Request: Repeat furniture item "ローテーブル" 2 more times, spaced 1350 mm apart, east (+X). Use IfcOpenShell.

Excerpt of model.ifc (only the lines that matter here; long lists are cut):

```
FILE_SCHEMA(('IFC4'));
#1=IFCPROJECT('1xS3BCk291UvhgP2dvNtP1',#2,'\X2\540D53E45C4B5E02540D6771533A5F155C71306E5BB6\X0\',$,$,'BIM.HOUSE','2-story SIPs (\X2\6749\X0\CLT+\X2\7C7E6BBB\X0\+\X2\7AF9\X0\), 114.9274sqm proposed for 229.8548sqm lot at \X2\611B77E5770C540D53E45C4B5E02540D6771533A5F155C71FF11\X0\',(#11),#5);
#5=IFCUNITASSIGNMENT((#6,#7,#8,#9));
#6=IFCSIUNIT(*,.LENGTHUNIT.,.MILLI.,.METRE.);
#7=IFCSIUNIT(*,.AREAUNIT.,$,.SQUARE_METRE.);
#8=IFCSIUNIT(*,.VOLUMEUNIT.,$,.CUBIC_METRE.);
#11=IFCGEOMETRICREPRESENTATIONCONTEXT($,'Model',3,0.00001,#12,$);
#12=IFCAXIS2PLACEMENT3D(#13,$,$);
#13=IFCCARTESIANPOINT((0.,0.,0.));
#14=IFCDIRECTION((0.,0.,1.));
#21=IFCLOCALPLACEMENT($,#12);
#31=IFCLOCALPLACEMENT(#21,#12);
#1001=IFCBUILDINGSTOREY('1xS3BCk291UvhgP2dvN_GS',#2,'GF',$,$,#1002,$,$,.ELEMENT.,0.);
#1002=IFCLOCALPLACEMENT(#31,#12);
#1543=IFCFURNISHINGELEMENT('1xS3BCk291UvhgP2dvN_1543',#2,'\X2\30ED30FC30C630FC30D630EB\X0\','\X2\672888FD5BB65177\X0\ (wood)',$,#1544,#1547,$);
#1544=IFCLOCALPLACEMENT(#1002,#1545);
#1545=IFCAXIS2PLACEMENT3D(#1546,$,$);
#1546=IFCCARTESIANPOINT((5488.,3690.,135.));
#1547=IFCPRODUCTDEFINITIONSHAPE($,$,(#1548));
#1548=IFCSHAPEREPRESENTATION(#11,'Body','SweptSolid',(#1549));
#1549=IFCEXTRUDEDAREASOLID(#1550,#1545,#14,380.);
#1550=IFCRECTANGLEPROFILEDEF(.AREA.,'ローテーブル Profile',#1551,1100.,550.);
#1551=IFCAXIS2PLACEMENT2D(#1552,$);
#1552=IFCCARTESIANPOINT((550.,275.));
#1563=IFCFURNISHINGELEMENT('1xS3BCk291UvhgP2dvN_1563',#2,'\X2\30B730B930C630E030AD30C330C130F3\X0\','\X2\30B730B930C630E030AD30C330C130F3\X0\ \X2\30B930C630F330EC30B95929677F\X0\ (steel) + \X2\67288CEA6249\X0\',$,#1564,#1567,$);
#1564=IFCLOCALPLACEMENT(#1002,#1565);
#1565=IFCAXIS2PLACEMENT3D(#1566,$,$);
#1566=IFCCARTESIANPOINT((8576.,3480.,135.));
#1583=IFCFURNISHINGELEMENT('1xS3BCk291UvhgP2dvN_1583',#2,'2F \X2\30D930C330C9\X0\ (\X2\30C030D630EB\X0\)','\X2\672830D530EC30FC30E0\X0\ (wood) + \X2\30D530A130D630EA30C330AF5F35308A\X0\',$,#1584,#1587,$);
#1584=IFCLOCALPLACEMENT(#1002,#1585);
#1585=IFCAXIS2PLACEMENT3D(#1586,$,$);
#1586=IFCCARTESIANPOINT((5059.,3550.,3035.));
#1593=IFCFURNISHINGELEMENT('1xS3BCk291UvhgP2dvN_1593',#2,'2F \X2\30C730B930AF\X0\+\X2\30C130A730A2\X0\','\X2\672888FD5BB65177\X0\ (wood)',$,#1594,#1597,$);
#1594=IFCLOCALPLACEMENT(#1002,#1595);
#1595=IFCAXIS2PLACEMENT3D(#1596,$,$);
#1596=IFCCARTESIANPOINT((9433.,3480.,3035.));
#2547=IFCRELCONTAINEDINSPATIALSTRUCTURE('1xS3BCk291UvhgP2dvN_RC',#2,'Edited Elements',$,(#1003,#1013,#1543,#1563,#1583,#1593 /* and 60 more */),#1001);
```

```python
import numpy as np
import ifcopenshell
import ifcopenshell.api.geometry
import ifcopenshell.api.root
import ifcopenshell.util.element
import ifcopenshell.util.placement

model = ifcopenshell.open("model.ifc")


def reuse_history(source, copy):
    """copy_class also copies each property set's owner history, people and application; keep the originals."""
    for rel in copy.IsDefinedBy:
        if rel.is_a("IfcRelDefinesByProperties") and (history := rel.RelatingPropertyDefinition.OwnerHistory):
            rel.RelatingPropertyDefinition.OwnerHistory = source.OwnerHistory
            ifcopenshell.util.element.remove_deep2(model, history)


source = model.by_id(1543)
base = ifcopenshell.util.placement.get_local_placement(source.ObjectPlacement)
step = np.array([1.0, 0.0, 0.0]) * 1350.0

for i in range(1, 3):
    copy = ifcopenshell.api.root.copy_class(model, product=source)
    copy.Representation = ifcopenshell.util.element.copy_deep(
        model, source.Representation, exclude=["IfcGeometricRepresentationContext", "IfcRepresentationMap"]
    )
    reuse_history(source, copy)
    matrix = base.copy()
    matrix[:3, 3] += i * step
    print("added at", matrix[:3, 3].round(3) + 0.0)
    ifcopenshell.api.geometry.edit_object_placement(model, product=copy, matrix=matrix, is_si=False)

model.write("model_updated.ifc")
```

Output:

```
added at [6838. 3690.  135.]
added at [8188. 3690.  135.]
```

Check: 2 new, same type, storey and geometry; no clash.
